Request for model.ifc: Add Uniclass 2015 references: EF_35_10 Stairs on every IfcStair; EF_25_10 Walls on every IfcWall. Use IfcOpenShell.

First a look at what the model holds.

```python
import ifcopenshell

model = ifcopenshell.open("model.ifc")
print(model.schema)
print("classifications:", [c.Name for c in model.by_type("IfcClassification")])
for ifc_class in ("IfcDoor", "IfcRoof", "IfcStair", "IfcWall", "IfcWindow"):
    print(ifc_class, len(model.by_type(ifc_class)))
```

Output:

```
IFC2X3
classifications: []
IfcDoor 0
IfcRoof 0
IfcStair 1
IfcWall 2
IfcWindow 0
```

```python
import ifcopenshell
import ifcopenshell.api.classification

model = ifcopenshell.open("model.ifc")

# IFC2X3 requires Source and Edition and has no link from the project to the system.
system = model.create_entity("IfcClassification", Source="NBS", Edition="2015", Name="Uniclass 2015")

codes = {
    "IfcStair": ("EF_35_10", "Stairs"),
    "IfcWall": ("EF_25_10", "Walls"),
}
for ifc_class, (code, name) in codes.items():
    products = model.by_type(ifc_class)
    ifcopenshell.api.classification.add_reference(
        model, products=products, classification=system, identification=code, name=name
    )
    print(code, len(products))

model.write("model_edited.ifc")
```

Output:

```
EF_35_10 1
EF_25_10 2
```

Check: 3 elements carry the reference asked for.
